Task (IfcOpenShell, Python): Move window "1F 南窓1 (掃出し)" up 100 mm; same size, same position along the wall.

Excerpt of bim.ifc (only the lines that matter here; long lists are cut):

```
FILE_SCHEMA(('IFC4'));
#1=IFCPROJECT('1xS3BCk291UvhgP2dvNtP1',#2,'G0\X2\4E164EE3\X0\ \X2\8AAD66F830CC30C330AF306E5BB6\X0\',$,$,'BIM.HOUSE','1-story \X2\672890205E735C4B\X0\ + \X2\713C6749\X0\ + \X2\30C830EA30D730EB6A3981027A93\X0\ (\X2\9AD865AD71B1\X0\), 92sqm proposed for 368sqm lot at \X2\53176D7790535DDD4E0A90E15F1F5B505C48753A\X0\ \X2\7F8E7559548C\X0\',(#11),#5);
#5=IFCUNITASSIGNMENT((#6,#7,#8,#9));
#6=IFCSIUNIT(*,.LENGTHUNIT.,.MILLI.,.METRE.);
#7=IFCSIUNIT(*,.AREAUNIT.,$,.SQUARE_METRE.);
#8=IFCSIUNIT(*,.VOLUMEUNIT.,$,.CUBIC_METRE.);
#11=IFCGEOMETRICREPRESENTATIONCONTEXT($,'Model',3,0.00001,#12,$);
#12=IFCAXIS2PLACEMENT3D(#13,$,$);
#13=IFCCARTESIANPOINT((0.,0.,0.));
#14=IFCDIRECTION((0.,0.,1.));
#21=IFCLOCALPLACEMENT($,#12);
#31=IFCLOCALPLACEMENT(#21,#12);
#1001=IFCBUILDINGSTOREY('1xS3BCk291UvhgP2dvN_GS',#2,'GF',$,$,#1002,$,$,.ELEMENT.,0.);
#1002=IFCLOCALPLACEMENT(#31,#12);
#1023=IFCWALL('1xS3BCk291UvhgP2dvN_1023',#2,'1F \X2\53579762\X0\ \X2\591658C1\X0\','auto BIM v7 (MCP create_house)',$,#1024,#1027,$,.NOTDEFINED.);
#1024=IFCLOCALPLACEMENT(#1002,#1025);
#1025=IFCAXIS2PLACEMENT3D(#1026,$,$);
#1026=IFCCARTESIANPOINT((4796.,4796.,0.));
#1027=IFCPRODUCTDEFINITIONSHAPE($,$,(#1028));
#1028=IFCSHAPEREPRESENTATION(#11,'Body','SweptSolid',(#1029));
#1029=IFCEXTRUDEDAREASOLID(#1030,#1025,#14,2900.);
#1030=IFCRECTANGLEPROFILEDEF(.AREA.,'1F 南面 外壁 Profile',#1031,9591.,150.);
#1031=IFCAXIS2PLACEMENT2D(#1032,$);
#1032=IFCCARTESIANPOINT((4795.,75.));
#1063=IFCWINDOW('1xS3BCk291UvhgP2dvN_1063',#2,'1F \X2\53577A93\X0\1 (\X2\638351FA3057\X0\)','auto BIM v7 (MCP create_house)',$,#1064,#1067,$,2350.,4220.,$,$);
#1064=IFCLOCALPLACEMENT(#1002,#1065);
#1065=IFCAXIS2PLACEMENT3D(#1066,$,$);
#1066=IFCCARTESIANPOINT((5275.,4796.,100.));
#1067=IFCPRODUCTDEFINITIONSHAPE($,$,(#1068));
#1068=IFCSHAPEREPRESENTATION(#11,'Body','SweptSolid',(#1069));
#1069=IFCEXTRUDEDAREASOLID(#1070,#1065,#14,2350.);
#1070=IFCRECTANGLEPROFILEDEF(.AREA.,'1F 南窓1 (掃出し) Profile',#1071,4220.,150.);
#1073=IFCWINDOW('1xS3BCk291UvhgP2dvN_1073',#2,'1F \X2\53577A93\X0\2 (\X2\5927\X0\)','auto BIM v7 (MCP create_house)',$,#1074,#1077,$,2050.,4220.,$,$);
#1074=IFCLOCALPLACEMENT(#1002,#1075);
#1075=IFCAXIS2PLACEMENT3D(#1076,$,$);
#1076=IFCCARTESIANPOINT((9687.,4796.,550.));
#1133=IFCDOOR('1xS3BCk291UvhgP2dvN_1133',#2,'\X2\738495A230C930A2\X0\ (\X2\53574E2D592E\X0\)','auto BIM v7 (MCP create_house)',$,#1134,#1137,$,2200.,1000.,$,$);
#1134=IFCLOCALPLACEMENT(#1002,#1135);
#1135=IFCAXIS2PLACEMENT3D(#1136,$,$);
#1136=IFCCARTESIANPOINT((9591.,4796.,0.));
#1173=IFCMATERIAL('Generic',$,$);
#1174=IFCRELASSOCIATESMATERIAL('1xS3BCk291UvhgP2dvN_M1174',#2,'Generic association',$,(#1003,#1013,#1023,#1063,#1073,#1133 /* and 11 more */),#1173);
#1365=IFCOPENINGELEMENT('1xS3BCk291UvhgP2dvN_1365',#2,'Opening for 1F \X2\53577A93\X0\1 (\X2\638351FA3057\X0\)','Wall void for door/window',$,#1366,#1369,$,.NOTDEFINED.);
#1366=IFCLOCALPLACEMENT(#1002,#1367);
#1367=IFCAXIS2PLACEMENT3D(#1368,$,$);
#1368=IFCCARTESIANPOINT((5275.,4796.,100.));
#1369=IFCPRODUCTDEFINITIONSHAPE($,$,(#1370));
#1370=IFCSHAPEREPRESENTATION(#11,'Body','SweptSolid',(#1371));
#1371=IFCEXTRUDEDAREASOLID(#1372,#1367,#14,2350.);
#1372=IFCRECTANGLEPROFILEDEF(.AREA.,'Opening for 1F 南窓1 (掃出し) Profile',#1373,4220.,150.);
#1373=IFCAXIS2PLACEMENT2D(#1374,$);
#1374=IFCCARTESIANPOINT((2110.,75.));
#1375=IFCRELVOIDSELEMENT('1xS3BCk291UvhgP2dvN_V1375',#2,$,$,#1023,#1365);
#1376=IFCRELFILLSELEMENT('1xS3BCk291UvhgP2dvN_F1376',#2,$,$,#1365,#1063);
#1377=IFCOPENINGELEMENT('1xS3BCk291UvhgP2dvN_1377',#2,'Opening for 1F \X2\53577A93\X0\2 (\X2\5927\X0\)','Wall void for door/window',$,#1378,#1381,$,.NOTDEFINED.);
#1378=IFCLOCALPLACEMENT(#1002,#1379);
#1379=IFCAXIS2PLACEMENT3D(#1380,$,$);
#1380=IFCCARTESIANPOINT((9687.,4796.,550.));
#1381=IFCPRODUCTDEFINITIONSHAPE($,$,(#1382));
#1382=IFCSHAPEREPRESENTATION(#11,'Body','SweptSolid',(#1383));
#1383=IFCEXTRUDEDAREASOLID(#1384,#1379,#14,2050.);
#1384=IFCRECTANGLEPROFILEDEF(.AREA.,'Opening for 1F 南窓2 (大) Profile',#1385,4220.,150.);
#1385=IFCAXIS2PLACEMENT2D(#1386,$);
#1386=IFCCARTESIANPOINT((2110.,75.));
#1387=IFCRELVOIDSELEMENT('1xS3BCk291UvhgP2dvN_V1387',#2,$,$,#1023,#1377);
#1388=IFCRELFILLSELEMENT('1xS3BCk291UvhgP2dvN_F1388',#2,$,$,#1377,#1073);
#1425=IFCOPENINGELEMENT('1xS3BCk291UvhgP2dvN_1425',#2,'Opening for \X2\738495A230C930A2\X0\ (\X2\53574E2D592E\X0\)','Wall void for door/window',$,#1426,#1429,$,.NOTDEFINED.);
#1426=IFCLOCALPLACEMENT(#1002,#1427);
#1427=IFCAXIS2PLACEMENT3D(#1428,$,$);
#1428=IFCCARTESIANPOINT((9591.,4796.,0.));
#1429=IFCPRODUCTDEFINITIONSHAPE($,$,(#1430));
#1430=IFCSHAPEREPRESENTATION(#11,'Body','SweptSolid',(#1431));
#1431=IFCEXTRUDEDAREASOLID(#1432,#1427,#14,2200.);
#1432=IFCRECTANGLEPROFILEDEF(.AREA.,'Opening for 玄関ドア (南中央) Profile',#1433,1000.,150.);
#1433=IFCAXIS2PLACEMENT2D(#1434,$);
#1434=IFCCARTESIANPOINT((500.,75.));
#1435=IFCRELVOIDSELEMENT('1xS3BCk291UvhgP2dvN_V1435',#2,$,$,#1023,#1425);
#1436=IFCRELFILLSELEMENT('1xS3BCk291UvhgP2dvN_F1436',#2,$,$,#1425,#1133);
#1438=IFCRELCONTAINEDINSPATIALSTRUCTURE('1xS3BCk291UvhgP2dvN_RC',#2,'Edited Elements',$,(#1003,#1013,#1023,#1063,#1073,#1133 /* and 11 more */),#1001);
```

```python
import numpy as np
import ifcopenshell
import ifcopenshell.api.geometry
import ifcopenshell.util.placement
import ifcopenshell.util.unit

model = ifcopenshell.open("bim.ifc")
unit_scale = ifcopenshell.util.unit.calculate_unit_scale(model)

window = model.by_id(1063)
opening = window.FillsVoids[0].RelatingOpeningElement
dz = 0.1 / unit_scale

shift = np.array([0.0, 0.0, dz])
# The window is not placed relative to its opening, so move both.
for product in (opening, window):
    matrix = ifcopenshell.util.placement.get_local_placement(product.ObjectPlacement)
    matrix[:3, 3] += shift
    ifcopenshell.api.geometry.edit_object_placement(model, product=product, matrix=matrix, is_si=False)

print(f"moved by {dz * unit_scale:+.3f} m")

model.write("bim_edited.ifc")
```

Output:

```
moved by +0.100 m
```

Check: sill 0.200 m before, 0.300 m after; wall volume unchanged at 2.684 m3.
